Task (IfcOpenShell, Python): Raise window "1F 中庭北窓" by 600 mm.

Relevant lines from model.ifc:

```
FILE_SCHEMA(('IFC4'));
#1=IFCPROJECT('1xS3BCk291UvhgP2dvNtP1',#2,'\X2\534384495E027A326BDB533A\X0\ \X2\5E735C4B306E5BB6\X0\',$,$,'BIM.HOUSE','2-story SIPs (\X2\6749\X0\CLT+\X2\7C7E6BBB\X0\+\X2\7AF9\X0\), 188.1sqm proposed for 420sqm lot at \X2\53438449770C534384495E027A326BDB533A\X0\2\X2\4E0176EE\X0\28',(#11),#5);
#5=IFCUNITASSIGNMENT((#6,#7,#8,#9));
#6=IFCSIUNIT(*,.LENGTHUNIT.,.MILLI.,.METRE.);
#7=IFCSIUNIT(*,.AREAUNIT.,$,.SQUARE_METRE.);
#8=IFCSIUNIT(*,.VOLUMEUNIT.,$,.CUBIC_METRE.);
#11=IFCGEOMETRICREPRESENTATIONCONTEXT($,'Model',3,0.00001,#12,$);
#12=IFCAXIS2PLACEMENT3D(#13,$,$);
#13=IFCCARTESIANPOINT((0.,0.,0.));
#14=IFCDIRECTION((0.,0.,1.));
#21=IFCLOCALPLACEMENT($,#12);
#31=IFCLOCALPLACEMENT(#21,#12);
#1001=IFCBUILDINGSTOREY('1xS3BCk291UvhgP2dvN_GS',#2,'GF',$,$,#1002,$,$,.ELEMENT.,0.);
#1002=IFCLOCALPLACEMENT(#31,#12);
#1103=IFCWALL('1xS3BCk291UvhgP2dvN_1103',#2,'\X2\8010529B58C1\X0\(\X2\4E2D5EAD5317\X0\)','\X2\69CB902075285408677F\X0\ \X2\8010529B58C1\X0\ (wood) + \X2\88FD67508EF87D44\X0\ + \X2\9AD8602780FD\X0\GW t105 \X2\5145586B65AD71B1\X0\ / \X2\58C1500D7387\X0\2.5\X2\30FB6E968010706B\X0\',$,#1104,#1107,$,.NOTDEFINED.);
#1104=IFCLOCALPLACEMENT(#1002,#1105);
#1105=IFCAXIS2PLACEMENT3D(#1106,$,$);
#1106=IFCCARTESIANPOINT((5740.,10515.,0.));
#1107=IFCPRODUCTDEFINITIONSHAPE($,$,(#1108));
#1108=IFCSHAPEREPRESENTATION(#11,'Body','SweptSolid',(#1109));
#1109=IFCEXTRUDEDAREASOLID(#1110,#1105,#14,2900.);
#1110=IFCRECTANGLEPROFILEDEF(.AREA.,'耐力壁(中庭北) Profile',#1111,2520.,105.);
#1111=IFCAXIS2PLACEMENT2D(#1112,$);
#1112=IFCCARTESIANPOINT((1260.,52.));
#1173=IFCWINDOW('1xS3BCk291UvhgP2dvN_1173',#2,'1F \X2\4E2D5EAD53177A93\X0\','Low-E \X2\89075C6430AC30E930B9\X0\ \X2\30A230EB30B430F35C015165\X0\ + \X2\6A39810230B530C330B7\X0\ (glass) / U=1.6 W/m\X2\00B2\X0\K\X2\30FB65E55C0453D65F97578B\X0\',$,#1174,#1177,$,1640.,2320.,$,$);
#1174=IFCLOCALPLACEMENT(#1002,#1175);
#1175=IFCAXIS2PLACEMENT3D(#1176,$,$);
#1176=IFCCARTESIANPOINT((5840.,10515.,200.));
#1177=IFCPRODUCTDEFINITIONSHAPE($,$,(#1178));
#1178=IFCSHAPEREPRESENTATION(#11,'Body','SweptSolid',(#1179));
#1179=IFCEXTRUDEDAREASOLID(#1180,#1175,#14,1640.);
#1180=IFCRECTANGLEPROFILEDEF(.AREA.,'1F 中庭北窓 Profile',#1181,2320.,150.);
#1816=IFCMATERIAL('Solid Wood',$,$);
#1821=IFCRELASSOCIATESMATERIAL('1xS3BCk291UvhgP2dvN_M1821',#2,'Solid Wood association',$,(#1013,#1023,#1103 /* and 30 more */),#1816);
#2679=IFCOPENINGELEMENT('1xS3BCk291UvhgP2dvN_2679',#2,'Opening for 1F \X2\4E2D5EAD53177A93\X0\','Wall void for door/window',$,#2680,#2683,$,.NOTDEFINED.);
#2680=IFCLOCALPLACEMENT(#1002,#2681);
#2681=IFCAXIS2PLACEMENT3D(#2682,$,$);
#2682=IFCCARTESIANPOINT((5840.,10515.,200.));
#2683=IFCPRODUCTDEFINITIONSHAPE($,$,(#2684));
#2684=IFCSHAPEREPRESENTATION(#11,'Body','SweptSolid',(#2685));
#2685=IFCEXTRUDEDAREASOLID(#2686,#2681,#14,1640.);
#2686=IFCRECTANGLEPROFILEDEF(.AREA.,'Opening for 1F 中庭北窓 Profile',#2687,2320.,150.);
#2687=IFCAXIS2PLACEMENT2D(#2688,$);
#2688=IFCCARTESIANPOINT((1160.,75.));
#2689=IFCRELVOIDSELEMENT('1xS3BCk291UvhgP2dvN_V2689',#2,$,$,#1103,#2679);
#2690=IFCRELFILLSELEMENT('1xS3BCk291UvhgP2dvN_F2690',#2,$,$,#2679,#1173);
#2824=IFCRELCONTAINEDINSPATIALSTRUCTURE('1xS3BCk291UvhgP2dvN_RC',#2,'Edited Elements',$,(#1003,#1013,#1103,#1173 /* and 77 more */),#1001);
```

```python
import numpy as np
import ifcopenshell
import ifcopenshell.api.geometry
import ifcopenshell.util.placement
import ifcopenshell.util.unit

model = ifcopenshell.open("model.ifc")
unit_scale = ifcopenshell.util.unit.calculate_unit_scale(model)

window = model.by_id(1173)
opening = window.FillsVoids[0].RelatingOpeningElement
dz = 600.0

shift = np.array([0.0, 0.0, dz])
# The window is not placed relative to its opening, so move both.
for product in (opening, window):
    matrix = ifcopenshell.util.placement.get_local_placement(product.ObjectPlacement)
    matrix[:3, 3] += shift
    ifcopenshell.api.geometry.edit_object_placement(model, product=product, matrix=matrix, is_si=False)

print(f"moved by {dz * unit_scale:+.3f} m")

model.write("model_edited.ifc")
```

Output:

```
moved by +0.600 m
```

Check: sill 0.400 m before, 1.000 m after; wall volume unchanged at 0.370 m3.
